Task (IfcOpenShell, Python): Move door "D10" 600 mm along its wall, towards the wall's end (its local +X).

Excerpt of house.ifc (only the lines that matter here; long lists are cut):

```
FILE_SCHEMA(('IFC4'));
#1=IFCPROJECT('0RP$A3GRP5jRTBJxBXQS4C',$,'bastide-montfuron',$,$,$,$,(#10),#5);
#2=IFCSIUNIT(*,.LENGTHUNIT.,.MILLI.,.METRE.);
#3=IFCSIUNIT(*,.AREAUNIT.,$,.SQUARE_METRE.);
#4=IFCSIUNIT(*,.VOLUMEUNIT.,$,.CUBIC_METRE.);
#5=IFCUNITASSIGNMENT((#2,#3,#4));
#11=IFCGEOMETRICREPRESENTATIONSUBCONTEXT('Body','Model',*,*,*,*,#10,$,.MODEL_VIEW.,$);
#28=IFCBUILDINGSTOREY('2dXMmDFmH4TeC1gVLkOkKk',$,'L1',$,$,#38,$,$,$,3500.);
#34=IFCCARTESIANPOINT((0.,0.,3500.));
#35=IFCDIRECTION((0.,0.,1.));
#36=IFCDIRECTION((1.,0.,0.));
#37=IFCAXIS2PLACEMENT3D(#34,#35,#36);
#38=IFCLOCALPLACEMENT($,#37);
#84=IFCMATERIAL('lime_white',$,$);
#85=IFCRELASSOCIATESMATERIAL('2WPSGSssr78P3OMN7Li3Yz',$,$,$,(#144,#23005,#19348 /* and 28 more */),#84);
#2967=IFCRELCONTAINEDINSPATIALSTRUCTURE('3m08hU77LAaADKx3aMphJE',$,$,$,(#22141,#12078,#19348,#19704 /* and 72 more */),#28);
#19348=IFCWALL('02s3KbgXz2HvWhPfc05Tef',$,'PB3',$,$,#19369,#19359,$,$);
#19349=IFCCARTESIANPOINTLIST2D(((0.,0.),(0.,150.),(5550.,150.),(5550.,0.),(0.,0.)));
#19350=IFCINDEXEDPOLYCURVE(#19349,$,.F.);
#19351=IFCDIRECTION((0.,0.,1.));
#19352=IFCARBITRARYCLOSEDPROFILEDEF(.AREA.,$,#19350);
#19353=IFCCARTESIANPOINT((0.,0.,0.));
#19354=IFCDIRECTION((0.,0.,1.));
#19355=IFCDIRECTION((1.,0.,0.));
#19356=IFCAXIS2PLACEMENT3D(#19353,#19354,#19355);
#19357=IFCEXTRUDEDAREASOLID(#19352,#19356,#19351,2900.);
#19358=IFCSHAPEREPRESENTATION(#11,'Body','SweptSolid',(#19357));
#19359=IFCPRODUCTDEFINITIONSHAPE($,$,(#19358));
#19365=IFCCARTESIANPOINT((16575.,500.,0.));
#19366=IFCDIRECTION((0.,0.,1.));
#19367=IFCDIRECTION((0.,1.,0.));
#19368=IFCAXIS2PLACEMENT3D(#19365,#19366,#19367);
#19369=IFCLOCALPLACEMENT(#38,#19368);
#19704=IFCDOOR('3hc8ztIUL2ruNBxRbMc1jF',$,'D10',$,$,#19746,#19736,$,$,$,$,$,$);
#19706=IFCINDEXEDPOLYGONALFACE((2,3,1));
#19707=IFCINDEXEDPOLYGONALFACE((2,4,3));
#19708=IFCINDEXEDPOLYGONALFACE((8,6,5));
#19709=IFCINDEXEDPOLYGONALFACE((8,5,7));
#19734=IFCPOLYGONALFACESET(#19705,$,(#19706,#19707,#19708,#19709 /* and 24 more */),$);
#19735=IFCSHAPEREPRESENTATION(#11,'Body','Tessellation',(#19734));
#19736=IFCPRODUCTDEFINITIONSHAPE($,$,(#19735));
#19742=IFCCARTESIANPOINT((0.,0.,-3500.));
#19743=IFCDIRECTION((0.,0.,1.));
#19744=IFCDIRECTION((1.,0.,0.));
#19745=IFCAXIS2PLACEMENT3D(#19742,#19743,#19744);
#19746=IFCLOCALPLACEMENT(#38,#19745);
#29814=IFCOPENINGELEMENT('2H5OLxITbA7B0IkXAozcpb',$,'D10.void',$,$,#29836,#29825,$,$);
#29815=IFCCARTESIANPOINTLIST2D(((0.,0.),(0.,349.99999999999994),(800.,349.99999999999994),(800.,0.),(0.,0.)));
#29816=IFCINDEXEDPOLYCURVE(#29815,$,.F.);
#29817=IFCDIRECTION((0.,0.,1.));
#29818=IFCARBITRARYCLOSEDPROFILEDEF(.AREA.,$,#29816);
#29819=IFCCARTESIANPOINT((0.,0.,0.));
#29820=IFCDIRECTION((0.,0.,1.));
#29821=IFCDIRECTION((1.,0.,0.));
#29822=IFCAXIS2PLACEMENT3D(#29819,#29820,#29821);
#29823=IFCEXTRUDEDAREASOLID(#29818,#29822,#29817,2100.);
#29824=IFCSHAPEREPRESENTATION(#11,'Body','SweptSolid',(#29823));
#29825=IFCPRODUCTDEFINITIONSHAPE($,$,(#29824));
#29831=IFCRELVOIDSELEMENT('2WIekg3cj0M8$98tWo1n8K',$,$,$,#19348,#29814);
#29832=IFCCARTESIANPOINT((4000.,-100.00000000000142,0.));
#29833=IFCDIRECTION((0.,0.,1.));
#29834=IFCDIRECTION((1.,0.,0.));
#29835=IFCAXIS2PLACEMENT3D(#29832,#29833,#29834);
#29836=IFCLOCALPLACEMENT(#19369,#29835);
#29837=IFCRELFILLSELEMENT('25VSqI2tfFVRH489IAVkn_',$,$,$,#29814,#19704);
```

```python
import ifcopenshell
import ifcopenshell.api.geometry
import ifcopenshell.util.placement

model = ifcopenshell.open("house.ifc")

door = model.by_id(19704)
opening = door.FillsVoids[0].RelatingOpeningElement
wall = opening.VoidsElements[0].RelatingBuildingElement

wall_matrix = ifcopenshell.util.placement.get_local_placement(wall.ObjectPlacement)
shift = wall_matrix[:3, 0] * 600.0
before = ifcopenshell.util.placement.get_local_placement(door.ObjectPlacement)[:3, 3].copy()

# The door is not placed relative to its opening, so move both.
for product in (opening, door):
    matrix = ifcopenshell.util.placement.get_local_placement(product.ObjectPlacement)
    matrix[:3, 3] += shift
    ifcopenshell.api.geometry.edit_object_placement(model, product=product, matrix=matrix, is_si=False)

after = ifcopenshell.util.placement.get_local_placement(door.ObjectPlacement)[:3, 3]
print("door moved by", (after - before).round(3) + 0.0)

model.write("house-out.ifc")
```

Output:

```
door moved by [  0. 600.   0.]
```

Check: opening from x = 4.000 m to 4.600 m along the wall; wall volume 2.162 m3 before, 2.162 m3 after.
